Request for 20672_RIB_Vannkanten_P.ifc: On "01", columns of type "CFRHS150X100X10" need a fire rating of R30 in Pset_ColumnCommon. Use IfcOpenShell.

First a look at what the model holds.

```python
import ifcopenshell
import ifcopenshell.util.element

model = ifcopenshell.open("20672_RIB_Vannkanten_P.ifc")
print(model.schema)
storey = next(s for s in model.by_type("IfcBuildingStorey") if s.Name == "01")
columns = [e for e in ifcopenshell.util.element.get_decomposition(storey) if e.is_a("IfcColumn")]
seen = {}
for e in columns:
    element_type = ifcopenshell.util.element.get_type(e)
    key = (element_type.Name if element_type != e and element_type else None, ifcopenshell.util.element.get_pset(e, "Pset_ColumnCommon", "FireRating"))
    seen[key] = seen.get(key, 0) + 1
for (name, value), count in sorted(seen.items(), key=str):
    print(count, "x", name, "|", value)
```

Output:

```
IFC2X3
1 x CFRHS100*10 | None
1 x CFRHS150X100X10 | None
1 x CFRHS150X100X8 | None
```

```python
import ifcopenshell
import ifcopenshell.api.pset
import ifcopenshell.util.element

model = ifcopenshell.open("20672_RIB_Vannkanten_P.ifc")

storey = next(s for s in model.by_type("IfcBuildingStorey") if s.Name == "01")
columns = [e for e in ifcopenshell.util.element.get_decomposition(storey) if e.is_a("IfcColumn")]

count = 0
for e in columns:
    element_type = ifcopenshell.util.element.get_type(e)
    if element_type in (None, e) or element_type.Name != "CFRHS150X100X10":
        continue
    # add_pset returns the element's existing set when there is one.
    pset = ifcopenshell.api.pset.add_pset(model, product=e, name="Pset_ColumnCommon")
    ifcopenshell.api.pset.edit_pset(model, pset=pset, properties={"FireRating": "R30"})
    count += 1

print(count, "columns updated")

model.write("20672_RIB_Vannkanten_P_edited.ifc")
```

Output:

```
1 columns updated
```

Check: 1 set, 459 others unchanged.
